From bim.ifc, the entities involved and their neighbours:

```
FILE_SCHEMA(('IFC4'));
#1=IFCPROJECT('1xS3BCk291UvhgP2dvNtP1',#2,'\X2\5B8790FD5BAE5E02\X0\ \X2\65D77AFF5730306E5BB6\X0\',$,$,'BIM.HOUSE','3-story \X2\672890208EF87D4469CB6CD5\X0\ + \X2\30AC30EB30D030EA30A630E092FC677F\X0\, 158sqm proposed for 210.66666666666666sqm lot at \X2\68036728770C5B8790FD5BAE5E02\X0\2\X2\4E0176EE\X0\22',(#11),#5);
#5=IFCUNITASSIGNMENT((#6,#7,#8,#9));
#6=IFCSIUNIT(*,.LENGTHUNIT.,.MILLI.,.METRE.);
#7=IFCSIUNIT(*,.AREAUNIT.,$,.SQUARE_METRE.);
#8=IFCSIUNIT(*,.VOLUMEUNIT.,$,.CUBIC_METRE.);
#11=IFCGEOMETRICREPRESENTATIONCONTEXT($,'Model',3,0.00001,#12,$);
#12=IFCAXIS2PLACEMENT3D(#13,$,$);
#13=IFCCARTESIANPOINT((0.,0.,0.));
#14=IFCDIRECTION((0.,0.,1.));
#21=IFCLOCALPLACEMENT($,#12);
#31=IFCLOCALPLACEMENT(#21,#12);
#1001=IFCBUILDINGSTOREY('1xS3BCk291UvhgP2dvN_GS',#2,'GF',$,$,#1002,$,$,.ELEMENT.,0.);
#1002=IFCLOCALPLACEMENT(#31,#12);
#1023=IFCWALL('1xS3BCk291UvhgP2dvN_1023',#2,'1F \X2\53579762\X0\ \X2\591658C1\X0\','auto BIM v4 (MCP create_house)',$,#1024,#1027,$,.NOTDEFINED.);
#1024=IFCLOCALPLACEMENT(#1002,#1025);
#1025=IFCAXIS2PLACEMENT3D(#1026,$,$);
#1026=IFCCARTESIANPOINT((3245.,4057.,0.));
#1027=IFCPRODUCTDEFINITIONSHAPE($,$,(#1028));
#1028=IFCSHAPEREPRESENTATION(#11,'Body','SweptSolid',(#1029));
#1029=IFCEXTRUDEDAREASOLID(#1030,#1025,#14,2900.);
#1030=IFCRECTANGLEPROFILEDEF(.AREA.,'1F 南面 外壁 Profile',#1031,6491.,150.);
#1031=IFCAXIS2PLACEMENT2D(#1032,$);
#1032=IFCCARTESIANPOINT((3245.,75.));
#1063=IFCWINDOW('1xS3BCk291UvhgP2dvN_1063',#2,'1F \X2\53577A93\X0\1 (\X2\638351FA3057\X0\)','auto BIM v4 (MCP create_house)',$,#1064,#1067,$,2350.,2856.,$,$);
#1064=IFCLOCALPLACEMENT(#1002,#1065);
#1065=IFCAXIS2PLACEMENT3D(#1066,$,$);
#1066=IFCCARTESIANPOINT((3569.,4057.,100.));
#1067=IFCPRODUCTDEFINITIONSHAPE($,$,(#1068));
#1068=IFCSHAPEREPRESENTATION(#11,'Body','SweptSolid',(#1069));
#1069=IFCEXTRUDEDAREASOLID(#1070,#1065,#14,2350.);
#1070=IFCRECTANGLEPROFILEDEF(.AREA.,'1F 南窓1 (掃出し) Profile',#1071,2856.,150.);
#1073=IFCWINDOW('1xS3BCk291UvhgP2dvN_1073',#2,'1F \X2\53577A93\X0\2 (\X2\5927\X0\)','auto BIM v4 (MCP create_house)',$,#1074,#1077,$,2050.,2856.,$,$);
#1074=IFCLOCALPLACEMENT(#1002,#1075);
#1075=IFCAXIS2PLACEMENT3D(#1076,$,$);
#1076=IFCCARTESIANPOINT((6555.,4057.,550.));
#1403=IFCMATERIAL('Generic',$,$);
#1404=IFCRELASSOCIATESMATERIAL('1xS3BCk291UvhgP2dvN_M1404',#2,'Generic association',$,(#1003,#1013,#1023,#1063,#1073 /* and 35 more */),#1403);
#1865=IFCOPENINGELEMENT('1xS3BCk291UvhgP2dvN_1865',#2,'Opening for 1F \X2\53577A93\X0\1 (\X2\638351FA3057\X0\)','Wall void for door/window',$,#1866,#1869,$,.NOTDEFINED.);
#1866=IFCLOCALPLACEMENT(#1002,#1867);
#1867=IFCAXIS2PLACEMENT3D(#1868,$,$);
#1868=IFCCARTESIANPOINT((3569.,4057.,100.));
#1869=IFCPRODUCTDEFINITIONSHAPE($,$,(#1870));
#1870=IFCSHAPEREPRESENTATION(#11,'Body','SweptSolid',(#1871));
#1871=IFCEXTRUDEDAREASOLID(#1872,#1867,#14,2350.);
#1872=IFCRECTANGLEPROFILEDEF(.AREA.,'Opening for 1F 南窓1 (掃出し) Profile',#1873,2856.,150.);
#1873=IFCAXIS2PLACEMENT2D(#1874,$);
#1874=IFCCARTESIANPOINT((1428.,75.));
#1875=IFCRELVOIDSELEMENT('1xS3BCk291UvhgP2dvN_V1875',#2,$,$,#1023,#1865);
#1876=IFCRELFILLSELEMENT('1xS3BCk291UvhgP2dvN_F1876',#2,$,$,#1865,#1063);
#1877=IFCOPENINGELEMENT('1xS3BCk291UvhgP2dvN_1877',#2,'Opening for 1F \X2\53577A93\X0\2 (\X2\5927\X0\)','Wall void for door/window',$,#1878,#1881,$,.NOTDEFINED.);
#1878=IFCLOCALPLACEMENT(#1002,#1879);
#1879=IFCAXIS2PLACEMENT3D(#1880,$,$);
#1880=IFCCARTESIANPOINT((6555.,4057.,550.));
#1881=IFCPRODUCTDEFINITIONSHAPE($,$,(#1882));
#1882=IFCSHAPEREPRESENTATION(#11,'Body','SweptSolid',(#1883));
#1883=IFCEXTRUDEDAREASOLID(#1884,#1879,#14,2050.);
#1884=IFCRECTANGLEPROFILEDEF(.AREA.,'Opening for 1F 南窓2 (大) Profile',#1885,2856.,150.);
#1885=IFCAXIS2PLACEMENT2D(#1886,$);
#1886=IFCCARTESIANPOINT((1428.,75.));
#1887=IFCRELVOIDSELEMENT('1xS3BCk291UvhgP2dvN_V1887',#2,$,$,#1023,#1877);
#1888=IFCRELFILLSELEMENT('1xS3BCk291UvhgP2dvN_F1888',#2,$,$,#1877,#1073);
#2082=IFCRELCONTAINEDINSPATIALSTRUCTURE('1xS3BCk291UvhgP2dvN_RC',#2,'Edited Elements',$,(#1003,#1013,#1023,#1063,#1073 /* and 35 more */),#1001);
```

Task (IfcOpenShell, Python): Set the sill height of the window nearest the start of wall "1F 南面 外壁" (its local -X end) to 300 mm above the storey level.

```python
import numpy as np
import ifcopenshell
import ifcopenshell.api.geometry
import ifcopenshell.geom
import ifcopenshell.util.element
import ifcopenshell.util.placement
import ifcopenshell.util.shape
import ifcopenshell.util.unit

model = ifcopenshell.open("bim.ifc")
unit_scale = ifcopenshell.util.unit.calculate_unit_scale(model)

window = model.by_guid("1xS3BCk291UvhgP2dvN_1063")
opening = window.FillsVoids[0].RelatingOpeningElement
storey = ifcopenshell.util.element.get_container(window, ifc_class="IfcBuildingStorey")
level = ifcopenshell.util.placement.get_local_placement(storey.ObjectPlacement)[2, 3]

# The opening's origin need not be at the sill, so measure its lowest point.
shape = ifcopenshell.geom.create_shape(ifcopenshell.geom.settings(), opening)
bottom = ifcopenshell.util.shape.get_shape_bottom_elevation(shape, shape.geometry) / unit_scale
dz = level + 0.3 / unit_scale - bottom

shift = np.array([0.0, 0.0, dz])
# The window is not placed relative to its opening, so move both.
for product in (opening, window):
    matrix = ifcopenshell.util.placement.get_local_placement(product.ObjectPlacement)
    matrix[:3, 3] += shift
    ifcopenshell.api.geometry.edit_object_placement(model, product=product, matrix=matrix, is_si=False)

print(f"moved by {dz * unit_scale:+.3f} m")

model.write("bim_v2.ifc")
```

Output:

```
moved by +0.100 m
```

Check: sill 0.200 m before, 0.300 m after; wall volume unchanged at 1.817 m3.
